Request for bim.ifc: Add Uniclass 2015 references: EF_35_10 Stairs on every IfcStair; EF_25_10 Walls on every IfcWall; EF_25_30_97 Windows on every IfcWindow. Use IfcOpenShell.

First a look at what the model holds.

```python
import ifcopenshell

model = ifcopenshell.open("bim.ifc")
print(model.schema)
print("classifications:", [c.Name for c in model.by_type("IfcClassification")])
for ifc_class in ("IfcDoor", "IfcRoof", "IfcStair", "IfcWall", "IfcWindow"):
    print(ifc_class, len(model.by_type(ifc_class)))
```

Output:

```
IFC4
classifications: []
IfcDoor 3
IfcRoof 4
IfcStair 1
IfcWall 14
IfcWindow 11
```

```python
import ifcopenshell
import ifcopenshell.api.classification

model = ifcopenshell.open("bim.ifc")

system = ifcopenshell.api.classification.add_classification(model, classification="Uniclass 2015")

codes = {
    "IfcStair": ("EF_35_10", "Stairs"),
    "IfcWall": ("EF_25_10", "Walls"),
    "IfcWindow": ("EF_25_30_97", "Windows"),
}
for ifc_class, (code, name) in codes.items():
    products = model.by_type(ifc_class)
    ifcopenshell.api.classification.add_reference(
        model, products=products, classification=system, identification=code, name=name
    )
    print(code, len(products))

model.write("bim-out.ifc")
```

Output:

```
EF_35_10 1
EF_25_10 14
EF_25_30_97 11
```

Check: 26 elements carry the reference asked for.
